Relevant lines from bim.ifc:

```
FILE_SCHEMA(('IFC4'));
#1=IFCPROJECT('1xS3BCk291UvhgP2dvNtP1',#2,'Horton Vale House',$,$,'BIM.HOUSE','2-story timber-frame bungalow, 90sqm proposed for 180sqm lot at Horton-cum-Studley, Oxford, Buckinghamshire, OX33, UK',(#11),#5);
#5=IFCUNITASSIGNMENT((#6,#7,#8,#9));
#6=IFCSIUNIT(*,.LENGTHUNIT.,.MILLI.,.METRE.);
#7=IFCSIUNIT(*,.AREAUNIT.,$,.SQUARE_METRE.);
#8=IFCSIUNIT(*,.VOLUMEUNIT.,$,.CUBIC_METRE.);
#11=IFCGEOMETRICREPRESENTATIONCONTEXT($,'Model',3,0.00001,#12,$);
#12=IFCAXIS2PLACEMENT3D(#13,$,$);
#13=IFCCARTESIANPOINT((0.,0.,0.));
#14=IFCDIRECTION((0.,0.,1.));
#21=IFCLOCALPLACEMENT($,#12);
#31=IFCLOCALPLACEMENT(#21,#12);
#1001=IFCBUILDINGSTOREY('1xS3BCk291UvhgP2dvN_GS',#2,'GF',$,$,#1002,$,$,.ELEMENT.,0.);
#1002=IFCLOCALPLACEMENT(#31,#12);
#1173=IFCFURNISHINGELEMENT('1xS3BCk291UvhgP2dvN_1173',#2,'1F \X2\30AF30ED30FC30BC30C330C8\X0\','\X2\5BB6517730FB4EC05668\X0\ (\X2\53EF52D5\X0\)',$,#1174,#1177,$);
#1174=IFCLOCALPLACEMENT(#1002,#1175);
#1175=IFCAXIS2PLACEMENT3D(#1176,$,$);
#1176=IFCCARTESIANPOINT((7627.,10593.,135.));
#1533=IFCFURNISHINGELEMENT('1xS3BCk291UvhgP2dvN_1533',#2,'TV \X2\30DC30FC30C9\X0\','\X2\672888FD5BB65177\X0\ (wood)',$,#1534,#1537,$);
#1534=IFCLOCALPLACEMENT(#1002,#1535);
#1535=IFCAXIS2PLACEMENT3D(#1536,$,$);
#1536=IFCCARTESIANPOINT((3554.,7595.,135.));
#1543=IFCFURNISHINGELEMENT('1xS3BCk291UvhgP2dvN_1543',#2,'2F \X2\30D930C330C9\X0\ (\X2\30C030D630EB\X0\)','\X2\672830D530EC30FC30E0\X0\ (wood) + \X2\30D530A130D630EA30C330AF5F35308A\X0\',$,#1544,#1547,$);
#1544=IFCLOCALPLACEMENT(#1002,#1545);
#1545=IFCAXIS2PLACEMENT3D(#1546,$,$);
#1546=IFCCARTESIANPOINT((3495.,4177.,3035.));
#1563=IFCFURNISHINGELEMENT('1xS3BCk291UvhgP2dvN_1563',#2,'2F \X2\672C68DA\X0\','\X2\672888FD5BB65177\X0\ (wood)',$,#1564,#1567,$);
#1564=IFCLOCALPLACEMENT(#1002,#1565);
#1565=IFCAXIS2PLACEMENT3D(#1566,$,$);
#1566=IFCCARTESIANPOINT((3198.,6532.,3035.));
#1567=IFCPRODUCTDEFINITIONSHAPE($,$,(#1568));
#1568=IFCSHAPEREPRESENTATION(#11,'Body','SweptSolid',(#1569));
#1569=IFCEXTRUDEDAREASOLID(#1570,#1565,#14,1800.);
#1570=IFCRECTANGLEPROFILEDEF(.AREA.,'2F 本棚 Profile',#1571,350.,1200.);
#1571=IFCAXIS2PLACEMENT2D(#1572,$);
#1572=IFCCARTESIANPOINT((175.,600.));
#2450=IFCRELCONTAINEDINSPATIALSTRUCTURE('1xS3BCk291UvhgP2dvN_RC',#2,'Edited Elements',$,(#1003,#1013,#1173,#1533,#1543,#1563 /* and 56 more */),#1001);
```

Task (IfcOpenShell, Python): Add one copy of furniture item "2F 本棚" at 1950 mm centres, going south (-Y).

```python
import numpy as np
import ifcopenshell
import ifcopenshell.api.geometry
import ifcopenshell.api.root
import ifcopenshell.util.element
import ifcopenshell.util.placement

model = ifcopenshell.open("bim.ifc")


def reuse_history(source, copy):
    """copy_class also copies each property set's owner history, people and application; keep the originals."""
    for rel in copy.IsDefinedBy:
        if rel.is_a("IfcRelDefinesByProperties") and (history := rel.RelatingPropertyDefinition.OwnerHistory):
            rel.RelatingPropertyDefinition.OwnerHistory = source.OwnerHistory
            ifcopenshell.util.element.remove_deep2(model, history)


source = model.by_id(1563)
base = ifcopenshell.util.placement.get_local_placement(source.ObjectPlacement)
step = np.array([0.0, -1.0, 0.0]) * 1950.0

for i in range(1, 2):
    copy = ifcopenshell.api.root.copy_class(model, product=source)
    copy.Representation = ifcopenshell.util.element.copy_deep(
        model, source.Representation, exclude=["IfcGeometricRepresentationContext", "IfcRepresentationMap"]
    )
    reuse_history(source, copy)
    matrix = base.copy()
    matrix[:3, 3] += i * step
    print("added at", matrix[:3, 3].round(3) + 0.0)
    ifcopenshell.api.geometry.edit_object_placement(model, product=copy, matrix=matrix, is_si=False)

model.write("bim_updated.ifc")
```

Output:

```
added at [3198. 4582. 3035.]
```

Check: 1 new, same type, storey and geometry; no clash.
